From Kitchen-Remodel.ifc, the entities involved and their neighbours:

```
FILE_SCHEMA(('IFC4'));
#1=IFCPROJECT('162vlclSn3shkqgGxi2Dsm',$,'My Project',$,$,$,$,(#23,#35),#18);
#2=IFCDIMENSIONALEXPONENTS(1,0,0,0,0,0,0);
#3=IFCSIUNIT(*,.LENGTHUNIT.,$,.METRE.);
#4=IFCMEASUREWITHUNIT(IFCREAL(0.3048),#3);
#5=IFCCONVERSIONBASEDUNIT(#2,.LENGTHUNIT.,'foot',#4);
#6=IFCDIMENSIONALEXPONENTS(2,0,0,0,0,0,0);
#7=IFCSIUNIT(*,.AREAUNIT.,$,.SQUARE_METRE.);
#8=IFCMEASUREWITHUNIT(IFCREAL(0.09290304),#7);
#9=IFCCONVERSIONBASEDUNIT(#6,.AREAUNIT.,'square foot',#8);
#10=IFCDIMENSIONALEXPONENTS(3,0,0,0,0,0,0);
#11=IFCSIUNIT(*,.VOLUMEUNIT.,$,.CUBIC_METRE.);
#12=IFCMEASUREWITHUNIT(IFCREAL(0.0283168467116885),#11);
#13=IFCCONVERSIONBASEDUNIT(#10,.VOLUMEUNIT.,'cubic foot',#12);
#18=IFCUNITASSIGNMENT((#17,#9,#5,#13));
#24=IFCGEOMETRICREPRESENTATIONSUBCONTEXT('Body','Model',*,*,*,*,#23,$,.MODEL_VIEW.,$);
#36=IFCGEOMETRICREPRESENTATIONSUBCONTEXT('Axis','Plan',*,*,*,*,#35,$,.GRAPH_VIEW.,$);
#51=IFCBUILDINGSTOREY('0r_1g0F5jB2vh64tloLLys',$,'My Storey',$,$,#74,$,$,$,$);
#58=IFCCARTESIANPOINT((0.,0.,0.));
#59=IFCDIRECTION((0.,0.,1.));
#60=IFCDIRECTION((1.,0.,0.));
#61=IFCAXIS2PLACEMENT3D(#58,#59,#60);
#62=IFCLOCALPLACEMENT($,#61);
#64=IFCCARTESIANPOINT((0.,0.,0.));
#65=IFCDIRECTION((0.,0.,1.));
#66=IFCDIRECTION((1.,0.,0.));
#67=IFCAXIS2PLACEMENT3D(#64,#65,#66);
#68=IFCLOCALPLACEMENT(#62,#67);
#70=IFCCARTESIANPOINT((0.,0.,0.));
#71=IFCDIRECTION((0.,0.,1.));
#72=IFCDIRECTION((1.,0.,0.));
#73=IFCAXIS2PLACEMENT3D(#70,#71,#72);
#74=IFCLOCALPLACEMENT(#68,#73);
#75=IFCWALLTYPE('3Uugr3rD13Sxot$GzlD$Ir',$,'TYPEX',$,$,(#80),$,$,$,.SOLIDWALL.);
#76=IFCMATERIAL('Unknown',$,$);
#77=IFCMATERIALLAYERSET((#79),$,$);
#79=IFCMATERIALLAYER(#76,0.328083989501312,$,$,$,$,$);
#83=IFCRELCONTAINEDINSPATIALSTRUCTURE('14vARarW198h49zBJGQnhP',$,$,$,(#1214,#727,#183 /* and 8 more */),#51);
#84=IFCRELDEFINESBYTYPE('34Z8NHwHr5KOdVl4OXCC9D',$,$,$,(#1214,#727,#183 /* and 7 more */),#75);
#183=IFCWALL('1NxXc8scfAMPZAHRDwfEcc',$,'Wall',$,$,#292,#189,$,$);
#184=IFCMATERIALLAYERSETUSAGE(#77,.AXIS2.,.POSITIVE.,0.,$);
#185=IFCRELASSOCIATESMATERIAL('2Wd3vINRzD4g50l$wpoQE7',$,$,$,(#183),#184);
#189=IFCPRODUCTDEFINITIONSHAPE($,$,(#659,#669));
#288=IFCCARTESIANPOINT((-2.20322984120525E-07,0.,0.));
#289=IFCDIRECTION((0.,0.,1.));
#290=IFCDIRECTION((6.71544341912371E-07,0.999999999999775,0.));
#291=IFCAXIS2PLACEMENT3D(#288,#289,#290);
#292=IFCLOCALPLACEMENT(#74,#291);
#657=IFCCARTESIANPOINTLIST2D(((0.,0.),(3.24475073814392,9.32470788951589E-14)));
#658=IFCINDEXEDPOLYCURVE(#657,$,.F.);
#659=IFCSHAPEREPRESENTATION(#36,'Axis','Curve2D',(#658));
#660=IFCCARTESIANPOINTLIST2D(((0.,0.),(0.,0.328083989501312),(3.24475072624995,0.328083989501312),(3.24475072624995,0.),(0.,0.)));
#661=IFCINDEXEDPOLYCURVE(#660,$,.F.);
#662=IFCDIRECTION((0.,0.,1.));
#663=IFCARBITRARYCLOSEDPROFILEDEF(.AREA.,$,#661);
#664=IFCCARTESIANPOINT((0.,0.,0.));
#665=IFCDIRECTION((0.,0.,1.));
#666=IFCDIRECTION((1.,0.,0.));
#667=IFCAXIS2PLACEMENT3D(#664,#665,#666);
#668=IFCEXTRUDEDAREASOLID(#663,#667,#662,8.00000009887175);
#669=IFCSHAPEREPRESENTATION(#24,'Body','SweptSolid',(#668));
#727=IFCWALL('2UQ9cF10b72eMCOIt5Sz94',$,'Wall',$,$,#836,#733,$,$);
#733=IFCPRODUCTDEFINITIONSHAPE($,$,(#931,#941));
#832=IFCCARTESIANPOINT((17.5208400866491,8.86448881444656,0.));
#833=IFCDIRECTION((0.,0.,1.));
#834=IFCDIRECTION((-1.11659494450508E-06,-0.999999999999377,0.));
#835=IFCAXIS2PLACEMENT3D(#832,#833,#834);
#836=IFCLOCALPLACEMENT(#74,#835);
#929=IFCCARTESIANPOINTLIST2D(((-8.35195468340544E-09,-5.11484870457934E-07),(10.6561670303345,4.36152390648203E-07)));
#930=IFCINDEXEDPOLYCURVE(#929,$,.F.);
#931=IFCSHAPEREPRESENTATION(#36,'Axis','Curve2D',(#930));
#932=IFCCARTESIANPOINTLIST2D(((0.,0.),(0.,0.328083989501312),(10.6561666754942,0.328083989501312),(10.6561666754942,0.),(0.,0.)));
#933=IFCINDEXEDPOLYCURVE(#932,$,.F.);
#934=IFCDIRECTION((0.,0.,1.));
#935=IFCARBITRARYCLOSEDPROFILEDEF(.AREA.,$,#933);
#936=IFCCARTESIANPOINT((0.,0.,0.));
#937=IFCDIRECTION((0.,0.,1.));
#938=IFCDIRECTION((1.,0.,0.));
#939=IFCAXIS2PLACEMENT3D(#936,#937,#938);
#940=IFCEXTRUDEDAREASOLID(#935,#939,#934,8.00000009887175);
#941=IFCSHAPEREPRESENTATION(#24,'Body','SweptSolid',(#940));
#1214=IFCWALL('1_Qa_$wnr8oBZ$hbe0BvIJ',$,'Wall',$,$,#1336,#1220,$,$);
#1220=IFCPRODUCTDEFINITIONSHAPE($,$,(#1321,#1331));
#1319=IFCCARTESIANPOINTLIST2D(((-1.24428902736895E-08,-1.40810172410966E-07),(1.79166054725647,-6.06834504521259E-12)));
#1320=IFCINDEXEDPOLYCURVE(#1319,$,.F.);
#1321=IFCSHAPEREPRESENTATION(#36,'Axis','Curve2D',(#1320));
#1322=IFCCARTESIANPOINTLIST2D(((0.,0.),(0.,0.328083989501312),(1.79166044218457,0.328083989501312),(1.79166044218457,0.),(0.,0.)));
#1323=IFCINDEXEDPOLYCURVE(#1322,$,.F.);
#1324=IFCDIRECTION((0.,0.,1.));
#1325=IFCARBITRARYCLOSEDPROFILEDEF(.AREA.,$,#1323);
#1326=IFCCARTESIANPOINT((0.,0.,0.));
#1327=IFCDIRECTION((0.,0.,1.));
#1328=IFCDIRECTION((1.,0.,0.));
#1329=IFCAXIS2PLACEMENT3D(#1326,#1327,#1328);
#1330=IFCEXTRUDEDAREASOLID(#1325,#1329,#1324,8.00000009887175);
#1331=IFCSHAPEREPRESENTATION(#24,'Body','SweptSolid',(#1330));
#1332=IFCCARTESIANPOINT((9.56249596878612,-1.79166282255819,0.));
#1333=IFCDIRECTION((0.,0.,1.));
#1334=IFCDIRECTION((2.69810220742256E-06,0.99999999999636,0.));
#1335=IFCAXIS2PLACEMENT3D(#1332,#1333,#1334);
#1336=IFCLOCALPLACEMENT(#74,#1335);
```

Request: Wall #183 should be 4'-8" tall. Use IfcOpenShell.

```python
import ifcopenshell
import ifcopenshell.geom
import ifcopenshell.util.representation
import ifcopenshell.util.shape
import ifcopenshell.util.unit

model = ifcopenshell.open("Kitchen-Remodel.ifc")
unit_scale = ifcopenshell.util.unit.calculate_unit_scale(model)
settings = ifcopenshell.geom.settings()


def volume(element):
    """Net volume in cubic metres, openings subtracted."""
    shape = ifcopenshell.geom.create_shape(settings, element)
    return ifcopenshell.util.shape.get_volume(shape.geometry)


wall = model.by_guid("1NxXc8scfAMPZAHRDwfEcc")
before = volume(wall)

body = ifcopenshell.util.representation.get_representation(wall, "Model", "Body")
solid = body.Items[0]
old_height = solid.Depth
solid.Depth = 56 * 0.0254 / unit_scale
after = volume(wall)

print(f"height {old_height:g} -> {solid.Depth:g}, volume {before:.3f} -> {after:.3f} m3")

model.write("Kitchen-Remodel_updated.ifc")
```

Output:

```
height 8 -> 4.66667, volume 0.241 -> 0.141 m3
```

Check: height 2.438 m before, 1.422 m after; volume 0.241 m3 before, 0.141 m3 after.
